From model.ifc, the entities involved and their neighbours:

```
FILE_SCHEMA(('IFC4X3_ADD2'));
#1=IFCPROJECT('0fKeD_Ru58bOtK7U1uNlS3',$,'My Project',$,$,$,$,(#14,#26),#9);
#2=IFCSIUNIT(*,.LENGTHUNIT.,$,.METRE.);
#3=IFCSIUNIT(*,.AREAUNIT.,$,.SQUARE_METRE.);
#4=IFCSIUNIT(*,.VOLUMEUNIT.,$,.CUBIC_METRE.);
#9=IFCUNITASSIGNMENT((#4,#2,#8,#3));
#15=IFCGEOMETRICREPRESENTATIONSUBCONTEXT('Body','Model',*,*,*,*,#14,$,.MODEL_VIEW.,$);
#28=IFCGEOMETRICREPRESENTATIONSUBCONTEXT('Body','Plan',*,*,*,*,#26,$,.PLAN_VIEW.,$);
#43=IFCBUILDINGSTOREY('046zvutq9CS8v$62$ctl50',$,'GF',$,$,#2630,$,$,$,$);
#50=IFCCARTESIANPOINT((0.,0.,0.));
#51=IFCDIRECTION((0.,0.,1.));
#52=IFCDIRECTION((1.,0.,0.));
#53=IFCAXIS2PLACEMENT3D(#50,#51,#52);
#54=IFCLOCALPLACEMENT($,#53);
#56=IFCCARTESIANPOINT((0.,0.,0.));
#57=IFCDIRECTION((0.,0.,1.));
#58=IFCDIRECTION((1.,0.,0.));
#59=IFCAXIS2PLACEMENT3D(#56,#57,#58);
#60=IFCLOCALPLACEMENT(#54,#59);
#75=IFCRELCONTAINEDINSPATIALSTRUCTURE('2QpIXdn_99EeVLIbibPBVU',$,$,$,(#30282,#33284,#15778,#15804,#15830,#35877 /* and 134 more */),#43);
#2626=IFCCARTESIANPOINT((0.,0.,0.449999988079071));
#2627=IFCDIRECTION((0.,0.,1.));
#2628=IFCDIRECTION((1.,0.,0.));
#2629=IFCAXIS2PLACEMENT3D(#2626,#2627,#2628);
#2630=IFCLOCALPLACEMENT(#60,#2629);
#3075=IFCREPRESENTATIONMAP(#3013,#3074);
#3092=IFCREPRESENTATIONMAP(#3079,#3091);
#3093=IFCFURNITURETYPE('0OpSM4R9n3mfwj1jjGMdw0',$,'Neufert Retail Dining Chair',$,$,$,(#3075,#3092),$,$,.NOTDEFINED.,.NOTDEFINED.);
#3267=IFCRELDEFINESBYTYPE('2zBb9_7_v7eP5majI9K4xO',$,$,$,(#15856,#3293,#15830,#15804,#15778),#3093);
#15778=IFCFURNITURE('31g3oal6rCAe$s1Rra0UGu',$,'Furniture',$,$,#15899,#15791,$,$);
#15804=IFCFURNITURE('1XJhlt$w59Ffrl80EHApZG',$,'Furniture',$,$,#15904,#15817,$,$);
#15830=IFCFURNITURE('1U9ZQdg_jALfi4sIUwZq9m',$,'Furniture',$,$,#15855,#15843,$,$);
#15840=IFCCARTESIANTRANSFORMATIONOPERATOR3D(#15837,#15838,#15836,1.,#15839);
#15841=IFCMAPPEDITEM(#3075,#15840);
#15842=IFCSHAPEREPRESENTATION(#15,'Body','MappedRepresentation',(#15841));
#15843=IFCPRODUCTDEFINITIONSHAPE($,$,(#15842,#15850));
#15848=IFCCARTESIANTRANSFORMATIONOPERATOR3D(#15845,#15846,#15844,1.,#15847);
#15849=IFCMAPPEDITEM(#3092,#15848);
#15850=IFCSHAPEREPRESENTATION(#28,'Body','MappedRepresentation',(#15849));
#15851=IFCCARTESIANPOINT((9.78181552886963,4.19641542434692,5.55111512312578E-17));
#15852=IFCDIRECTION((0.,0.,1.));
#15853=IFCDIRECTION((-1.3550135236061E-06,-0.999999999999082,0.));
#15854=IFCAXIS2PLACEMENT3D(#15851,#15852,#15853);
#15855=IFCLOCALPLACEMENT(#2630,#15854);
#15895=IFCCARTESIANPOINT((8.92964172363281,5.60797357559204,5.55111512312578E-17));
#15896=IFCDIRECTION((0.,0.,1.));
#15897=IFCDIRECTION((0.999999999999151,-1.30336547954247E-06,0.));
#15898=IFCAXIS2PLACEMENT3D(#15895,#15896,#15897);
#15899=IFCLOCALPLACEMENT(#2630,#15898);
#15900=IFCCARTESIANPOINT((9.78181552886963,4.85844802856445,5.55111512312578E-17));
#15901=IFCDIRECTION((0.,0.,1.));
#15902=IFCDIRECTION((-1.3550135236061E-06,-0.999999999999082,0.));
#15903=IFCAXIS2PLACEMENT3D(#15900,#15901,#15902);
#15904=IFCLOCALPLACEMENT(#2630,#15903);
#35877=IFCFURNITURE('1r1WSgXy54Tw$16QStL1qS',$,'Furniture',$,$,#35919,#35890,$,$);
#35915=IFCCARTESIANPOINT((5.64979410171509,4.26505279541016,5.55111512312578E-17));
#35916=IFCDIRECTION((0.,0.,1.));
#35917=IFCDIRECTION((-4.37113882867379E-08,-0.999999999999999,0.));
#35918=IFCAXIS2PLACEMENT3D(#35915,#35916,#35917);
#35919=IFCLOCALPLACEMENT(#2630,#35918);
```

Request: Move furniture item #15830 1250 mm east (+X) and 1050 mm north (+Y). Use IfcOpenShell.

```python
import ifcopenshell
import ifcopenshell.api.geometry
import ifcopenshell.util.placement

model = ifcopenshell.open("model.ifc")

item = model.by_id(15830)
matrix = ifcopenshell.util.placement.get_local_placement(item.ObjectPlacement)
matrix[0, 3] += 1.25
matrix[1, 3] += 1.05
ifcopenshell.api.geometry.edit_object_placement(model, product=item, matrix=matrix, is_si=False)

print(ifcopenshell.util.placement.get_local_placement(item.ObjectPlacement).round(3) + 0.0)

model.write("model_v2.ifc")
```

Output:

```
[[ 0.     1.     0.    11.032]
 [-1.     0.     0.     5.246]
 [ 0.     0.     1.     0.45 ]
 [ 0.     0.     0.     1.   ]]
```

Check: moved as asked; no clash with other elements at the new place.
